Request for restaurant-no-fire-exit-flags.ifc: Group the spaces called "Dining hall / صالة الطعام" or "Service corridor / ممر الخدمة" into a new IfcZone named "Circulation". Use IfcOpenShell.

First a look at what the model holds.

```python
import ifcopenshell

model = ifcopenshell.open("restaurant-no-fire-exit-flags.ifc")
print(model.schema)
seen = {}
for space in model.by_type("IfcSpace"):
    seen[space.LongName] = seen.get(space.LongName, 0) + 1
for name, count in sorted(seen.items(), key=str):
    print(count, "x", name)
print("zones:", [z.Name for z in model.by_type("IfcZone")][:20])
```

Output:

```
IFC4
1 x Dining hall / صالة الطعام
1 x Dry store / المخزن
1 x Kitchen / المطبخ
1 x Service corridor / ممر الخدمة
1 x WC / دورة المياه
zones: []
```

```python
import ifcopenshell
import ifcopenshell.api.group
import ifcopenshell.api.root

model = ifcopenshell.open("restaurant-no-fire-exit-flags.ifc")

names = {"Dining hall / صالة الطعام", "Service corridor / ممر الخدمة"}
spaces = [s for s in model.by_type("IfcSpace") if s.LongName in names]

zone = ifcopenshell.api.root.create_entity(model, ifc_class="IfcZone", name="Circulation")
ifcopenshell.api.group.assign_group(model, products=spaces, group=zone)
print(len(spaces), "spaces in", zone.Name)

model.write("restaurant-no-fire-exit-flags_updated.ifc")
```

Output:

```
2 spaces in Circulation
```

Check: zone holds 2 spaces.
